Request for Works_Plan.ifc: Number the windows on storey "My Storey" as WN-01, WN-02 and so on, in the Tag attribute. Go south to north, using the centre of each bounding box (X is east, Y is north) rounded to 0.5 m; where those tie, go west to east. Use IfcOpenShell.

First a look at what the model holds.

```python
import ifcopenshell
import ifcopenshell.util.element
import ifcopenshell.util.placement

model = ifcopenshell.open("Works_Plan.ifc")
print(model.schema)
storey = next(s for s in model.by_type("IfcBuildingStorey") if s.Name == "My Storey")
windows = [e for e in ifcopenshell.util.element.get_decomposition(storey) if e.is_a("IfcWindow")]
for e in sorted(windows, key=lambda e: e.id()):
    origin = ifcopenshell.util.placement.get_local_placement(e.ObjectPlacement)[:3, 3]
    print(e.id(), e.Tag, e.Name, origin.round(2) + 0.0, sep=" | ")
```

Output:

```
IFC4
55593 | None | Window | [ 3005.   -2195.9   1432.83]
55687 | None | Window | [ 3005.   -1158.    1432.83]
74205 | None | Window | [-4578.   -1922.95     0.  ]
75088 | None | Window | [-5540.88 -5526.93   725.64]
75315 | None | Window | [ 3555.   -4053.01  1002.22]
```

```python
import ifcopenshell
import ifcopenshell.geom
import ifcopenshell.util.element
import ifcopenshell.util.shape

model = ifcopenshell.open("Works_Plan.ifc")
settings = ifcopenshell.geom.settings()
settings.set("use-world-coords", True)


def centre(element):
    shape = ifcopenshell.geom.create_shape(settings, element)
    return ifcopenshell.util.shape.get_bbox_centroid(shape.geometry)


storey = next(s for s in model.by_type("IfcBuildingStorey") if s.Name == "My Storey")
windows = [e for e in ifcopenshell.util.element.get_decomposition(storey) if e.is_a("IfcWindow")]

# Insertion points can sit at a corner or the storey origin, so sort by the geometry (in metres).
centres = {e: centre(e) for e in windows}
windows.sort(key=lambda e: (round(centres[e][1] / 0.5), centres[e][0]))

for i, e in enumerate(windows, start=1):
    number = f"WN-{i:02d}"
    e.Tag = number
    print(e.id(), number)

model.write("Works_Plan_v2.ifc")
```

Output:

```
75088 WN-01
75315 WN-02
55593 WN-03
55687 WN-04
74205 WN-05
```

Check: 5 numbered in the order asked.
